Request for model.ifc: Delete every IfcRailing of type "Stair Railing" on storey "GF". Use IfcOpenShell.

First a look at what the model holds.

```python
import ifcopenshell
import ifcopenshell.util.element

model = ifcopenshell.open("model.ifc")
print(model.schema)
storey = next(s for s in model.by_type("IfcBuildingStorey") if s.Name == "GF")
railings = [e for e in ifcopenshell.util.element.get_decomposition(storey) if e.is_a("IfcRailing")]
seen = {}
for e in railings:
    element_type = ifcopenshell.util.element.get_type(e)
    name = element_type.Name if element_type not in (None, e) else None
    seen[name] = seen.get(name, 0) + 1
for name, count in sorted(seen.items(), key=str):
    print(count, "x", name)
```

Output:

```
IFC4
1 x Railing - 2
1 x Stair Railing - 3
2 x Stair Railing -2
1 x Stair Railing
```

```python
import ifcopenshell
import ifcopenshell.api.root
import ifcopenshell.util.element

model = ifcopenshell.open("model.ifc")

storey = next(s for s in model.by_type("IfcBuildingStorey") if s.Name == "GF")
railings = [e for e in ifcopenshell.util.element.get_decomposition(storey) if e.is_a("IfcRailing")]
targets = [e for e in railings if (t := ifcopenshell.util.element.get_type(e)) not in (None, e) and t.Name == "Stair Railing"]

for e in targets:
    ifcopenshell.api.root.remove_product(model, product=e)
print(len(targets), "removed")

model.write("model_rev.ifc")
```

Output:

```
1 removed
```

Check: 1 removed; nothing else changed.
